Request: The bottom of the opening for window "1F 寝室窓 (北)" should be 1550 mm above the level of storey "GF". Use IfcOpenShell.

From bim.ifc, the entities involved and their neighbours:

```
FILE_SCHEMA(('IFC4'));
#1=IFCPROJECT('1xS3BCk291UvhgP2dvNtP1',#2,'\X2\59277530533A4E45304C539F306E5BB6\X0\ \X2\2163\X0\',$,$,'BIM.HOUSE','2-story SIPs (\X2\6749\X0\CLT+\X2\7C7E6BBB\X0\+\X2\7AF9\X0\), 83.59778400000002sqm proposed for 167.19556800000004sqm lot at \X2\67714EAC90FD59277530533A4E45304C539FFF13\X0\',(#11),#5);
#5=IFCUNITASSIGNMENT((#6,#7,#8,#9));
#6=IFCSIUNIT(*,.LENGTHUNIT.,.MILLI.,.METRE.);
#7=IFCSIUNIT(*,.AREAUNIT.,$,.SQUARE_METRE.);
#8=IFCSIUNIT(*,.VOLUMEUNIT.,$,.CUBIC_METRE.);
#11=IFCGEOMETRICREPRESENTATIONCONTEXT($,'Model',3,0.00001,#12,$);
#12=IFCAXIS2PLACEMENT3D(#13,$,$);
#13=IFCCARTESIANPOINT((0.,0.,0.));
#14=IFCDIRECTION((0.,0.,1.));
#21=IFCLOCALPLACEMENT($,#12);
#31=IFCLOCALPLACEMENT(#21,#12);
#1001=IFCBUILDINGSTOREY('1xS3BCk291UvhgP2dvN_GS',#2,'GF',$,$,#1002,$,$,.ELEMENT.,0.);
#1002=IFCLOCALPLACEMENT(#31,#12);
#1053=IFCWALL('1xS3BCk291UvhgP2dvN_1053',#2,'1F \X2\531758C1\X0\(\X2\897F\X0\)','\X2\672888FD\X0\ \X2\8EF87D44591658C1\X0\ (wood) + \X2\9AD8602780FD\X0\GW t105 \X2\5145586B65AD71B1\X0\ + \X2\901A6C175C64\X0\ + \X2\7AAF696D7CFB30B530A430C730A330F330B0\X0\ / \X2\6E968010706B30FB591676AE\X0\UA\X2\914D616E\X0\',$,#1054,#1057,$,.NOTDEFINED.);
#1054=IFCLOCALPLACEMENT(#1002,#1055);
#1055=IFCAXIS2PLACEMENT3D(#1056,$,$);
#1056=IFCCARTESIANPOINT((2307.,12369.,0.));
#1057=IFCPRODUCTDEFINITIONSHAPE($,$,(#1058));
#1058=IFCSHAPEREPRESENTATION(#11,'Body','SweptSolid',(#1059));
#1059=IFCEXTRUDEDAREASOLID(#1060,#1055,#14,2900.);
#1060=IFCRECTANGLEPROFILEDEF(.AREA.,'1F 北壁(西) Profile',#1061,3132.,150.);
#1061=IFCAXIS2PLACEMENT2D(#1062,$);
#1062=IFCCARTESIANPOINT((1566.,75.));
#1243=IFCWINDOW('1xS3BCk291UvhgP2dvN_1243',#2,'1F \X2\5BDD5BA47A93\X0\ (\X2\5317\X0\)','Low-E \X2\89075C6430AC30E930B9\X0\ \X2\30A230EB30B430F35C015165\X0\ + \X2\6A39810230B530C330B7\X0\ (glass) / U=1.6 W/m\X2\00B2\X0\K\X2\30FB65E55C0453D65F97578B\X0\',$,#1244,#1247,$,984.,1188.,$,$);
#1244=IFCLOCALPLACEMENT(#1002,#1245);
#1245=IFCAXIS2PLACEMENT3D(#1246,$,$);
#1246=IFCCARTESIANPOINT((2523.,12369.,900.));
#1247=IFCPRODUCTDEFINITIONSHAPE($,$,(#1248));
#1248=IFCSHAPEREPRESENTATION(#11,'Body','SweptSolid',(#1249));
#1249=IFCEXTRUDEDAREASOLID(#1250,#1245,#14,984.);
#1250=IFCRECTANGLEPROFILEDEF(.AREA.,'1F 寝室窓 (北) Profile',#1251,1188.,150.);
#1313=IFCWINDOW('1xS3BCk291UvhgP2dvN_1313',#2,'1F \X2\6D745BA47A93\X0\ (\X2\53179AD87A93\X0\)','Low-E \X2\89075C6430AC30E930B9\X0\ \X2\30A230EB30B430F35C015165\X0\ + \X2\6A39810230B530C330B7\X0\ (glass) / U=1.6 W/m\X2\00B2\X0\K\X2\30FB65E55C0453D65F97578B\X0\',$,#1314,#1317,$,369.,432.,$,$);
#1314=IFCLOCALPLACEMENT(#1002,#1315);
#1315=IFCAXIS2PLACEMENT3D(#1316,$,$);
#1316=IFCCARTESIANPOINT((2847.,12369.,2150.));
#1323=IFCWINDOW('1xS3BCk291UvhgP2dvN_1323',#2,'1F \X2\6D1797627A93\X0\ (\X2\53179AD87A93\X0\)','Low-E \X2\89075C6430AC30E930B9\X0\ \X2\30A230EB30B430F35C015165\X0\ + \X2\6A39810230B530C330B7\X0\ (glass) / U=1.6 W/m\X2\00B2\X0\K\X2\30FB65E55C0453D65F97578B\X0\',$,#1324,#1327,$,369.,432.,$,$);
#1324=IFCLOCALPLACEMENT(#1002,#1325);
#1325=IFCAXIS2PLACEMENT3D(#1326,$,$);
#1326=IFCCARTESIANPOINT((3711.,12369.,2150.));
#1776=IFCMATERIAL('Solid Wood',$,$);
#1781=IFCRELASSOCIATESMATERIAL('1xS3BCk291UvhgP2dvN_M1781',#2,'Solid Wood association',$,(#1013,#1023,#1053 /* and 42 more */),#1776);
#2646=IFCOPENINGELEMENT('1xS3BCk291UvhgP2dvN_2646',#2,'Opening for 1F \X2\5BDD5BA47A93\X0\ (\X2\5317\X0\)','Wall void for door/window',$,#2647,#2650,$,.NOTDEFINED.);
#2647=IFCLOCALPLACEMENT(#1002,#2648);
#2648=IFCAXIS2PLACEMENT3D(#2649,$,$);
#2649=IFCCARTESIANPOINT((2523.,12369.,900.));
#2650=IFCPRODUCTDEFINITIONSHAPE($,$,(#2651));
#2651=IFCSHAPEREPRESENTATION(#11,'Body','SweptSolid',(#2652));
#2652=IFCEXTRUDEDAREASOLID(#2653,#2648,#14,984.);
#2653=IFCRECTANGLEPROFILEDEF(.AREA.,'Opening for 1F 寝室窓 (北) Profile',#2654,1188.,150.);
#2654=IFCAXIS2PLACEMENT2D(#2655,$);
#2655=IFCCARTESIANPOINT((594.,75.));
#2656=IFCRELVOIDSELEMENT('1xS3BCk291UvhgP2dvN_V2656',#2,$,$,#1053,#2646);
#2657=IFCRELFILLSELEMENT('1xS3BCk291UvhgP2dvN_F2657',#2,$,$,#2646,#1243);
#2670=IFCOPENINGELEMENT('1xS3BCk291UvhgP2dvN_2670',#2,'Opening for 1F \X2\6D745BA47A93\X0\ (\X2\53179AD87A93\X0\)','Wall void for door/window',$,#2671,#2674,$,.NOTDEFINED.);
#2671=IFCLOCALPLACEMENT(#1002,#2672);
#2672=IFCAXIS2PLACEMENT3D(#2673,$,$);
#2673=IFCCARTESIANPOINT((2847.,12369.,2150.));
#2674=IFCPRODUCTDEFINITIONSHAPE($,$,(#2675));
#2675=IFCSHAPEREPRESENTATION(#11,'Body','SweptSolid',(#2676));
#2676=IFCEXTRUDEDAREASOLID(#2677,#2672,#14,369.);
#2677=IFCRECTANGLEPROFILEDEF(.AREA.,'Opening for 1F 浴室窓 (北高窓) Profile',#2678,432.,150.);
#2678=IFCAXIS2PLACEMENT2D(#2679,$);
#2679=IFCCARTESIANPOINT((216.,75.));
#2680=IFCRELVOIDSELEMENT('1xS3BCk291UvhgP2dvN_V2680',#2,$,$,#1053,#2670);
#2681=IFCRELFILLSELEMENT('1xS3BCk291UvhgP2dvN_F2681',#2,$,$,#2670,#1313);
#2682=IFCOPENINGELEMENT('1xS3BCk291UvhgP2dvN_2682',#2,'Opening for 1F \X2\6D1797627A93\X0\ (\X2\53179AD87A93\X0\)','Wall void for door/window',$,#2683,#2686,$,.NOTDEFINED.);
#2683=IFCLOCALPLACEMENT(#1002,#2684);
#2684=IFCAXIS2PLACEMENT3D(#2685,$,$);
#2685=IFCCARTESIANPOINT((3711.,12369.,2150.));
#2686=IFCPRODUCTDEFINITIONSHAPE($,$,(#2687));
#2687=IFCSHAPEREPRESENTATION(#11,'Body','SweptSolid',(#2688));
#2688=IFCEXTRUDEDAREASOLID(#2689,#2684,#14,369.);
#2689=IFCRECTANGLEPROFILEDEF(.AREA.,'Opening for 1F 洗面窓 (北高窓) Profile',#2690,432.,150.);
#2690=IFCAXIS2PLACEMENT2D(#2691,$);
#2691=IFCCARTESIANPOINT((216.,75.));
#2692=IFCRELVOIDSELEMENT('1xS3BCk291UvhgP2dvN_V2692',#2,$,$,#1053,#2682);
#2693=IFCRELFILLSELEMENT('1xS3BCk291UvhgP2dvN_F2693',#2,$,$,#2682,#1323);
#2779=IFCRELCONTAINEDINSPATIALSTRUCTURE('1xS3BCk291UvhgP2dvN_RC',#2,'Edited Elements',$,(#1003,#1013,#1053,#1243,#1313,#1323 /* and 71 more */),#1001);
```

```python
import numpy as np
import ifcopenshell
import ifcopenshell.api.geometry
import ifcopenshell.geom
import ifcopenshell.util.element
import ifcopenshell.util.placement
import ifcopenshell.util.shape
import ifcopenshell.util.unit

model = ifcopenshell.open("bim.ifc")
unit_scale = ifcopenshell.util.unit.calculate_unit_scale(model)

window = model.by_guid("1xS3BCk291UvhgP2dvN_1243")
opening = window.FillsVoids[0].RelatingOpeningElement
storey = ifcopenshell.util.element.get_container(window, ifc_class="IfcBuildingStorey")
level = ifcopenshell.util.placement.get_local_placement(storey.ObjectPlacement)[2, 3]

# The opening's origin need not be at the sill, so measure its lowest point.
shape = ifcopenshell.geom.create_shape(ifcopenshell.geom.settings(), opening)
bottom = ifcopenshell.util.shape.get_shape_bottom_elevation(shape, shape.geometry) / unit_scale
dz = level + 1.55 / unit_scale - bottom

shift = np.array([0.0, 0.0, dz])
# The window is not placed relative to its opening, so move both.
for product in (opening, window):
    matrix = ifcopenshell.util.placement.get_local_placement(product.ObjectPlacement)
    matrix[:3, 3] += shift
    ifcopenshell.api.geometry.edit_object_placement(model, product=product, matrix=matrix, is_si=False)

print(f"moved by {dz * unit_scale:+.3f} m")

model.write("bim_rev.ifc")
```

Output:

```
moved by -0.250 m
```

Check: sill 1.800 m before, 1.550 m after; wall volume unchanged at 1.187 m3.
